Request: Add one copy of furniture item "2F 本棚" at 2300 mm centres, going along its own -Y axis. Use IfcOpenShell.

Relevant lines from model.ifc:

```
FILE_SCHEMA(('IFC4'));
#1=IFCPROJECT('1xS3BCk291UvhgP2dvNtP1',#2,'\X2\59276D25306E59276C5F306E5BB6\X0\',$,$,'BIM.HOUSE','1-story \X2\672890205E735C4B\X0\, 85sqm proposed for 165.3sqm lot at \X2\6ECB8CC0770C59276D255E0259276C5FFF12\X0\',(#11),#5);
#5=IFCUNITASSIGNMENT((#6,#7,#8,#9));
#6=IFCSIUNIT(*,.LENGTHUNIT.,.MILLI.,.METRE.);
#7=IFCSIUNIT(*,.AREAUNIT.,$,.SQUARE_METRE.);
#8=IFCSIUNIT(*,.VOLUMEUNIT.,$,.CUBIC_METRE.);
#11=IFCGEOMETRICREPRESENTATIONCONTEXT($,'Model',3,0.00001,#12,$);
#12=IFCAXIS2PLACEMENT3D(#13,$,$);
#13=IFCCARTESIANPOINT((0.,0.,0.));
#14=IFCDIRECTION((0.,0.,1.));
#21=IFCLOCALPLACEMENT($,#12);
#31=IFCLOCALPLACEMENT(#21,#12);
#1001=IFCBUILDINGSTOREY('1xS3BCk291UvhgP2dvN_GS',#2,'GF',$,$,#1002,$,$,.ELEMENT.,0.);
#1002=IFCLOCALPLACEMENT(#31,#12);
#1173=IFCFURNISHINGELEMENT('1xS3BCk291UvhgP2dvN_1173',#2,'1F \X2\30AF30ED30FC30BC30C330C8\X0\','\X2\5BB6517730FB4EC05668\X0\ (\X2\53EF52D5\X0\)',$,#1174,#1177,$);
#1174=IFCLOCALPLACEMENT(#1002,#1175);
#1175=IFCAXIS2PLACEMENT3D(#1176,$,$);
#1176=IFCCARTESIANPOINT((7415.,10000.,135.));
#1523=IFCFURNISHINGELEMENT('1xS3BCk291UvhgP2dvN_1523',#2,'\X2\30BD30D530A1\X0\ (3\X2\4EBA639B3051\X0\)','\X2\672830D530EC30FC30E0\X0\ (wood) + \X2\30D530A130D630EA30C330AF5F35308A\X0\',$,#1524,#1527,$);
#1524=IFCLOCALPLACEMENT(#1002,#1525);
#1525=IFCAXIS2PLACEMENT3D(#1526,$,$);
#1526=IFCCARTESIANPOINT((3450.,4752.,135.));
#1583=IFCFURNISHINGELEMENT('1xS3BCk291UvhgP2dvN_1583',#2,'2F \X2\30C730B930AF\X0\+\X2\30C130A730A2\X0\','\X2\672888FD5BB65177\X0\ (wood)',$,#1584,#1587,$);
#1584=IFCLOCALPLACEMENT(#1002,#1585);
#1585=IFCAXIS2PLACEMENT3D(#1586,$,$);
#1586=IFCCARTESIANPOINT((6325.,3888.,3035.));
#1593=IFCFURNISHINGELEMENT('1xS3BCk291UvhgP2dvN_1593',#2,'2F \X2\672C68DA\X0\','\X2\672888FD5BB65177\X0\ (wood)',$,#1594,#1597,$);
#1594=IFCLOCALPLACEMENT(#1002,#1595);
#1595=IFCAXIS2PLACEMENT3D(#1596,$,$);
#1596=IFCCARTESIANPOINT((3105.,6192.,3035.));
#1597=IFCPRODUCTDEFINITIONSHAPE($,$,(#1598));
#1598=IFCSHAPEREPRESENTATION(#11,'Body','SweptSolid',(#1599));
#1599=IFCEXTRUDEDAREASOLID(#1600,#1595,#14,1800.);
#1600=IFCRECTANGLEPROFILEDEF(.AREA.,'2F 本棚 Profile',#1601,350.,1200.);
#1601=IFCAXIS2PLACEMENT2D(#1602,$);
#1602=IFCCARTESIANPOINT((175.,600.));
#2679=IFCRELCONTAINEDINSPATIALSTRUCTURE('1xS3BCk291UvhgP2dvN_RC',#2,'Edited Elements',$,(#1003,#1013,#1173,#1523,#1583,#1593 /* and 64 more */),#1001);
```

```python
import ifcopenshell
import ifcopenshell.api.geometry
import ifcopenshell.api.root
import ifcopenshell.util.element
import ifcopenshell.util.placement

model = ifcopenshell.open("model.ifc")


def reuse_history(source, copy):
    """copy_class also copies each property set's owner history, people and application; keep the originals."""
    for rel in copy.IsDefinedBy:
        if rel.is_a("IfcRelDefinesByProperties") and (history := rel.RelatingPropertyDefinition.OwnerHistory):
            rel.RelatingPropertyDefinition.OwnerHistory = source.OwnerHistory
            ifcopenshell.util.element.remove_deep2(model, history)


source = model.by_id(1593)
base = ifcopenshell.util.placement.get_local_placement(source.ObjectPlacement)
step = -base[:3, 1] * 2300.0

for i in range(1, 2):
    copy = ifcopenshell.api.root.copy_class(model, product=source)
    copy.Representation = ifcopenshell.util.element.copy_deep(
        model, source.Representation, exclude=["IfcGeometricRepresentationContext", "IfcRepresentationMap"]
    )
    reuse_history(source, copy)
    matrix = base.copy()
    matrix[:3, 3] += i * step
    print("added at", matrix[:3, 3].round(3) + 0.0)
    ifcopenshell.api.geometry.edit_object_placement(model, product=copy, matrix=matrix, is_si=False)

model.write("model_v2.ifc")
```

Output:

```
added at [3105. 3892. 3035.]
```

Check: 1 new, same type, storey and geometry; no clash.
